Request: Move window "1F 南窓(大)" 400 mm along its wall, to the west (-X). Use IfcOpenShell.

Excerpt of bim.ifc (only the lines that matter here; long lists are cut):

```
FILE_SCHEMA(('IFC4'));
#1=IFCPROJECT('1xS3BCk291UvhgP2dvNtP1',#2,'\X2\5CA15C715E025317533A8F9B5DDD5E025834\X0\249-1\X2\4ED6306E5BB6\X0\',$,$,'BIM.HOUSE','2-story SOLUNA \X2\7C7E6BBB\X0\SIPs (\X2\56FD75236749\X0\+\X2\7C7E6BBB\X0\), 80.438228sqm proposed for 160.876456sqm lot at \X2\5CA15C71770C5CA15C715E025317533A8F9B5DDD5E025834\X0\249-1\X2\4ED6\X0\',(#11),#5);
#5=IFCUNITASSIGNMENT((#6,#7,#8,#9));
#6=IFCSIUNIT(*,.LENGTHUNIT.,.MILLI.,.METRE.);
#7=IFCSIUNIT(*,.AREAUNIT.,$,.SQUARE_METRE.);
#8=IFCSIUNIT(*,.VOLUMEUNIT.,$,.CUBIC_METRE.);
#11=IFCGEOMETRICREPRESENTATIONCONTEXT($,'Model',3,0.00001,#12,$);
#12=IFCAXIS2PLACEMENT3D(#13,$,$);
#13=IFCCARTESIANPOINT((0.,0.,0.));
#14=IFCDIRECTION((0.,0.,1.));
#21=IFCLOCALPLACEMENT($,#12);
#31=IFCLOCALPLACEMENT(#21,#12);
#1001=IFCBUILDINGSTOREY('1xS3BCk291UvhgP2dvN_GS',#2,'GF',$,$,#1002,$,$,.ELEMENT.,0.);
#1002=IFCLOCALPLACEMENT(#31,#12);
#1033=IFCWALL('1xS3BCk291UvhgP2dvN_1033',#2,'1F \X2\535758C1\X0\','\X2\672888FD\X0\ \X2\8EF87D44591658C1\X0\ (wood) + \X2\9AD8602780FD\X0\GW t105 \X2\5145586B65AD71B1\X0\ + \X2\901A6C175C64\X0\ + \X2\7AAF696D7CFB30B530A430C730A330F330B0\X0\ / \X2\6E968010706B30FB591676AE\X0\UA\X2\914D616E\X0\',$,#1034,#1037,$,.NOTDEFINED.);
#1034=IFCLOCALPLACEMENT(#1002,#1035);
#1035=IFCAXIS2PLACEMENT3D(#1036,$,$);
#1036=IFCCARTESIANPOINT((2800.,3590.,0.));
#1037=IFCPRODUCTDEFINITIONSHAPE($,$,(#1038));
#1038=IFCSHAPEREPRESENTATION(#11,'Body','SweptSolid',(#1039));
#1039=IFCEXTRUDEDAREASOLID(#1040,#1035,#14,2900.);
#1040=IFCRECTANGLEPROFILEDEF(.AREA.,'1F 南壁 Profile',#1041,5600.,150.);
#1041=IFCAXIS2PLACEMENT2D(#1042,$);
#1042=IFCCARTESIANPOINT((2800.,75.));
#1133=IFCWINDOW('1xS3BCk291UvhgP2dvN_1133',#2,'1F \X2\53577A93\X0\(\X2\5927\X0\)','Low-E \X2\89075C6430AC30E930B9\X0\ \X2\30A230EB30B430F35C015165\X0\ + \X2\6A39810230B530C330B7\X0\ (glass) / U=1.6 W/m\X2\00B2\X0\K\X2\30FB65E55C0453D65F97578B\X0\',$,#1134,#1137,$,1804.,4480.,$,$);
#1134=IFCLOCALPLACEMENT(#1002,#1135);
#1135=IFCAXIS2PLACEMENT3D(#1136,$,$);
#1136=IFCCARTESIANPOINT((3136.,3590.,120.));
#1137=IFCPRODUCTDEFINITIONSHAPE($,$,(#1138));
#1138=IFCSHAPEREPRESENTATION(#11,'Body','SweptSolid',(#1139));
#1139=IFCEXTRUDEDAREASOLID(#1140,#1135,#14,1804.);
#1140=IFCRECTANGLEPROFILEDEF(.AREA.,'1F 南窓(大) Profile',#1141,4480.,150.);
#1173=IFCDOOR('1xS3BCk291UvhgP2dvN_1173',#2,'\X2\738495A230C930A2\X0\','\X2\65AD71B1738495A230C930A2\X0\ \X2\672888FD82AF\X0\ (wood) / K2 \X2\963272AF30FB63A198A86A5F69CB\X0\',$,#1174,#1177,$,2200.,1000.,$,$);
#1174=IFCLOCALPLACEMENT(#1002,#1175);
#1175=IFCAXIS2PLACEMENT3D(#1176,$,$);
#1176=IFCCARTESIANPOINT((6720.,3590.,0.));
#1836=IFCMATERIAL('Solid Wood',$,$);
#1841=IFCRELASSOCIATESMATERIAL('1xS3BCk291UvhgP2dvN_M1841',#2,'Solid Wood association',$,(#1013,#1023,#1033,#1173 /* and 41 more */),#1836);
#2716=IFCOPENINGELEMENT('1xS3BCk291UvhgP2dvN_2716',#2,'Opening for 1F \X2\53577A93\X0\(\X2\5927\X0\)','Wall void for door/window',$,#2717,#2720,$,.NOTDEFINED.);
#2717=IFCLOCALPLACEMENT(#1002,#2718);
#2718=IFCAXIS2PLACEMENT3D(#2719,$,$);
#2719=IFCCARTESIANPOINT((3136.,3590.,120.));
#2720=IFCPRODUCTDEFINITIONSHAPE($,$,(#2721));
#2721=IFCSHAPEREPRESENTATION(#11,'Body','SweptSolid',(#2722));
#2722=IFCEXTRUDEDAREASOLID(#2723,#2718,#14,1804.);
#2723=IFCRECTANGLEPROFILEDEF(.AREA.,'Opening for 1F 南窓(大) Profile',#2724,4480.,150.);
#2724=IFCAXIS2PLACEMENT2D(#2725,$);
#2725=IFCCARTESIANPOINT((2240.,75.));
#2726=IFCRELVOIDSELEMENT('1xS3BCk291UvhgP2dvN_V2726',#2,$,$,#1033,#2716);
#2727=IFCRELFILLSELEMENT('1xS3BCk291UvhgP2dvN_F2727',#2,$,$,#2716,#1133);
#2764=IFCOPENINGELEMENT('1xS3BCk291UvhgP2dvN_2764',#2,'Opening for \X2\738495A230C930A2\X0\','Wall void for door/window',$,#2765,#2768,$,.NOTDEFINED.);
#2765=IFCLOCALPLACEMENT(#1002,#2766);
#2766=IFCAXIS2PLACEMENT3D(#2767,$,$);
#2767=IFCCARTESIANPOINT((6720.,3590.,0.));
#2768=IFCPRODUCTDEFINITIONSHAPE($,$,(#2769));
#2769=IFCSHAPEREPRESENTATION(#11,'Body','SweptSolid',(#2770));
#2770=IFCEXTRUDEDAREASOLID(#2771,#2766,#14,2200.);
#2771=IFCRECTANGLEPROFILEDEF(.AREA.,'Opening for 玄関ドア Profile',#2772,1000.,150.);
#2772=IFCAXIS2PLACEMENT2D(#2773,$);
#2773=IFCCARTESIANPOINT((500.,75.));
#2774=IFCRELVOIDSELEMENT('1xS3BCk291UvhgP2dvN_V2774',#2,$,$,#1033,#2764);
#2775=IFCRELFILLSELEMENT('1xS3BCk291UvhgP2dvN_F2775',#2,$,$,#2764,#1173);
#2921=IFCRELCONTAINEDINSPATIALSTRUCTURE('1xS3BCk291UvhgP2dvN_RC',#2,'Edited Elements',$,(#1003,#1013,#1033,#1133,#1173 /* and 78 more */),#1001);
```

```python
import ifcopenshell
import ifcopenshell.api.geometry
import ifcopenshell.util.placement
import ifcopenshell.util.unit

model = ifcopenshell.open("bim.ifc")
unit_scale = ifcopenshell.util.unit.calculate_unit_scale(model)

window = model.by_guid("1xS3BCk291UvhgP2dvN_1133")
opening = window.FillsVoids[0].RelatingOpeningElement
wall = opening.VoidsElements[0].RelatingBuildingElement

wall_matrix = ifcopenshell.util.placement.get_local_placement(wall.ObjectPlacement)
shift = wall_matrix[:3, 0] * -0.4 / unit_scale
before = ifcopenshell.util.placement.get_local_placement(window.ObjectPlacement)[:3, 3].copy()

# The window is not placed relative to its opening, so move both.
for product in (opening, window):
    matrix = ifcopenshell.util.placement.get_local_placement(product.ObjectPlacement)
    matrix[:3, 3] += shift
    ifcopenshell.api.geometry.edit_object_placement(model, product=product, matrix=matrix, is_si=False)

after = ifcopenshell.util.placement.get_local_placement(window.ObjectPlacement)[:3, 3]
print("window moved by", (after - before).round(3) + 0.0)

model.write("bim_v2.ifc")
```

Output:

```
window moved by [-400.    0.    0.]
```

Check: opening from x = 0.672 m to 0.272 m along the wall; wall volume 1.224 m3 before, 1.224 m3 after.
